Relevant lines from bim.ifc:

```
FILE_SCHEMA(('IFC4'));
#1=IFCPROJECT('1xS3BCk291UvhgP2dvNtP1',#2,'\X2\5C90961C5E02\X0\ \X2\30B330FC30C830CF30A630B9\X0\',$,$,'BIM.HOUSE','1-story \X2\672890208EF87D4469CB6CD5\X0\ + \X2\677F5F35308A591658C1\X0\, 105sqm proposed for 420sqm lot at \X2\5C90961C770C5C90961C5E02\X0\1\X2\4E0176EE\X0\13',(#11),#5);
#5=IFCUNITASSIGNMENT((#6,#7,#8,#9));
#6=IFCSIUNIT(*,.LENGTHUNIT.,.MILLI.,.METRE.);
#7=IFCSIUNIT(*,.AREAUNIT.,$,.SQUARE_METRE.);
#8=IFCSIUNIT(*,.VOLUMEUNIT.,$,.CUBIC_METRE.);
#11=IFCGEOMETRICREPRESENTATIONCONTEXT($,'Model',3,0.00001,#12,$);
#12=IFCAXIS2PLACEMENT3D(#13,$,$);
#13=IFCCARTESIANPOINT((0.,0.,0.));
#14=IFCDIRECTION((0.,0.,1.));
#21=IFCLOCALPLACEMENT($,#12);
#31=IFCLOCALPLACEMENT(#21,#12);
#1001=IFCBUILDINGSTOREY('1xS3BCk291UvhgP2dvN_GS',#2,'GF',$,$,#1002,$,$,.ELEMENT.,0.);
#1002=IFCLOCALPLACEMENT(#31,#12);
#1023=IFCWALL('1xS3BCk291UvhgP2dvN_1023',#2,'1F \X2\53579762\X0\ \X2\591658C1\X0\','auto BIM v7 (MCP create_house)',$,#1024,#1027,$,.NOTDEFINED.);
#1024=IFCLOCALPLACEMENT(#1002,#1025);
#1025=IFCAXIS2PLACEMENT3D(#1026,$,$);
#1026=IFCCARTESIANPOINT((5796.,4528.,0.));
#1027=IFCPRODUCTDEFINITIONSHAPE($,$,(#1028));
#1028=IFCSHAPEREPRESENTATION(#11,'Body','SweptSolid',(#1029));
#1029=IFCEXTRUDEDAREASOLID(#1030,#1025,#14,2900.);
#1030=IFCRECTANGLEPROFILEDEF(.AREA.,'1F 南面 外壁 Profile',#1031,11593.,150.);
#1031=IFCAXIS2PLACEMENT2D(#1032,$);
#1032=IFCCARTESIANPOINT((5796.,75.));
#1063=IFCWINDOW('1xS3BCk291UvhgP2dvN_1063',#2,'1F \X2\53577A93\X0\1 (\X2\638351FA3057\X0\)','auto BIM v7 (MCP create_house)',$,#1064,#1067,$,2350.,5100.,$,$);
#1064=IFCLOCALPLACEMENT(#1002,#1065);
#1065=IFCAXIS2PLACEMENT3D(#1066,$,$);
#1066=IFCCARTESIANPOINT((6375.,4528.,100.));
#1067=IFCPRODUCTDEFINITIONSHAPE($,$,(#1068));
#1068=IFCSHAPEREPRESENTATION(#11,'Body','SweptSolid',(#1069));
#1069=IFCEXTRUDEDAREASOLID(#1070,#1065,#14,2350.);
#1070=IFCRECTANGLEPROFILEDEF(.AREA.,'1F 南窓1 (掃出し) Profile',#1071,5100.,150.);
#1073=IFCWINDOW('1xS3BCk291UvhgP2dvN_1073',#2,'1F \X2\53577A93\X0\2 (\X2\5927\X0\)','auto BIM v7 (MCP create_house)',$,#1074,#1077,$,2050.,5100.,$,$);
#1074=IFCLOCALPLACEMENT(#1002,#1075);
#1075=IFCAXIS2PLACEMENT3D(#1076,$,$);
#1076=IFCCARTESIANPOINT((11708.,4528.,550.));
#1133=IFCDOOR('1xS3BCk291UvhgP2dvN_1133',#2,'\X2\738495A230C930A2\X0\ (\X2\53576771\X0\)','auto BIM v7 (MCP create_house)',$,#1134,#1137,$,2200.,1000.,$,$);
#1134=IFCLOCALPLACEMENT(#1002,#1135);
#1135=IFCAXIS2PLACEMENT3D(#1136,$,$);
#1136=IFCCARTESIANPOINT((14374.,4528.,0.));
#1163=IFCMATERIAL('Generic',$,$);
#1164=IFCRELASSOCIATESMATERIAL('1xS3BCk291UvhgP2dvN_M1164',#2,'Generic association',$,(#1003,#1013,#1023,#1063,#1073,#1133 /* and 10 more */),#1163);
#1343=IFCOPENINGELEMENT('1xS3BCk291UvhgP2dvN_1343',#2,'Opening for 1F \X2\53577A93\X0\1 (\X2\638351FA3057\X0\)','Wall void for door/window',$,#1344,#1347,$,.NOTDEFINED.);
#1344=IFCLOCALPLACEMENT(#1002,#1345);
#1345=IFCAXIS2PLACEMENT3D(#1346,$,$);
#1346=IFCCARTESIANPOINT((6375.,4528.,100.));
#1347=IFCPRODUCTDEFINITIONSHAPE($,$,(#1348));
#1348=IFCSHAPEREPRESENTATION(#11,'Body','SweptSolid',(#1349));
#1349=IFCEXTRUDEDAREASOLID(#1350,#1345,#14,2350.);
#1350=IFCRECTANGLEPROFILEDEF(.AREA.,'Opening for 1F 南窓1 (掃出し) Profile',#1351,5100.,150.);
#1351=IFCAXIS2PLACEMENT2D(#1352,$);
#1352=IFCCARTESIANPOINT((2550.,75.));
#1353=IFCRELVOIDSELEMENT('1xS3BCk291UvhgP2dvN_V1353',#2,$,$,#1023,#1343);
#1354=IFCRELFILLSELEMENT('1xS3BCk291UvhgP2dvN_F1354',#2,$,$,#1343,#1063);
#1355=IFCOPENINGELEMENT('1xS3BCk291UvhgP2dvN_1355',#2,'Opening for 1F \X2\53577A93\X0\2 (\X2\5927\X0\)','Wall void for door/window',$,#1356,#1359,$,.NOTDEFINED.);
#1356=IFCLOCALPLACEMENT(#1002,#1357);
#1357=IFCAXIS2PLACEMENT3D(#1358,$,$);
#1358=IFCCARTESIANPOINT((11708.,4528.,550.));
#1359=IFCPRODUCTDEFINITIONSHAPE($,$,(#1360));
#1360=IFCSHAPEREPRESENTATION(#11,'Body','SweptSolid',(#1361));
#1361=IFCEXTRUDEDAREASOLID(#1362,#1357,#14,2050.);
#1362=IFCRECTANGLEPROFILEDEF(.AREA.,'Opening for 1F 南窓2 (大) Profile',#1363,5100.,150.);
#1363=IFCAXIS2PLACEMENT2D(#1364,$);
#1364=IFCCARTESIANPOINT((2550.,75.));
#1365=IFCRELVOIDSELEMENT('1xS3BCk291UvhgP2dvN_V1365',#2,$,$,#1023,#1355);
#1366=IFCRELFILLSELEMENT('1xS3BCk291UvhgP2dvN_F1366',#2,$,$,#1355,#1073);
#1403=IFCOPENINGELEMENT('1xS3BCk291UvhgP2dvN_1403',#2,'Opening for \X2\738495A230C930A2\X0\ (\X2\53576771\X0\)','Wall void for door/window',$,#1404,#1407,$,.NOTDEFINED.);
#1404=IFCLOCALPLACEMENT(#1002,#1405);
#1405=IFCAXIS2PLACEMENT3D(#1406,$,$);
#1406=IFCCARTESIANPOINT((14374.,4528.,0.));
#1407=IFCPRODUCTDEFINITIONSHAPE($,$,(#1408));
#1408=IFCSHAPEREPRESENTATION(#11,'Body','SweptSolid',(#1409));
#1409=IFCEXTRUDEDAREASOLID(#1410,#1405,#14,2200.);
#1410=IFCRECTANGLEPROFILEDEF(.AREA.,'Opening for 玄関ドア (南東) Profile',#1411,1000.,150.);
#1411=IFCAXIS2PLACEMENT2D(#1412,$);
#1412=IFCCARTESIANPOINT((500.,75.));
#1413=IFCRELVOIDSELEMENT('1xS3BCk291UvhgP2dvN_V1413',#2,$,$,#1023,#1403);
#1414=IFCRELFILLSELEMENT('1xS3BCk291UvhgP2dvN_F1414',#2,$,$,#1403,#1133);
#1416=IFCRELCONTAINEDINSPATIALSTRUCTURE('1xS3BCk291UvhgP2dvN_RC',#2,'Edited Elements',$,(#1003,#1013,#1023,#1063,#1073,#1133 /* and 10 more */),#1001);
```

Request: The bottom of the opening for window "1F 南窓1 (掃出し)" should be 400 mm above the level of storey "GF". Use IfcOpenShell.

```python
import numpy as np
import ifcopenshell
import ifcopenshell.api.geometry
import ifcopenshell.geom
import ifcopenshell.util.element
import ifcopenshell.util.placement
import ifcopenshell.util.shape
import ifcopenshell.util.unit

model = ifcopenshell.open("bim.ifc")
unit_scale = ifcopenshell.util.unit.calculate_unit_scale(model)

window = model.by_guid("1xS3BCk291UvhgP2dvN_1063")
opening = window.FillsVoids[0].RelatingOpeningElement
storey = ifcopenshell.util.element.get_container(window, ifc_class="IfcBuildingStorey")
level = ifcopenshell.util.placement.get_local_placement(storey.ObjectPlacement)[2, 3]

# The opening's origin need not be at the sill, so measure its lowest point.
shape = ifcopenshell.geom.create_shape(ifcopenshell.geom.settings(), opening)
bottom = ifcopenshell.util.shape.get_shape_bottom_elevation(shape, shape.geometry) / unit_scale
dz = level + 400.0 - bottom

shift = np.array([0.0, 0.0, dz])
# The window is not placed relative to its opening, so move both.
for product in (opening, window):
    matrix = ifcopenshell.util.placement.get_local_placement(product.ObjectPlacement)
    matrix[:3, 3] += shift
    ifcopenshell.api.geometry.edit_object_placement(model, product=product, matrix=matrix, is_si=False)

print(f"moved by {dz * unit_scale:+.3f} m")

model.write("bim_updated.ifc")
```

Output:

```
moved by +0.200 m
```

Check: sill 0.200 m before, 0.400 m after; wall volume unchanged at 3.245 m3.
